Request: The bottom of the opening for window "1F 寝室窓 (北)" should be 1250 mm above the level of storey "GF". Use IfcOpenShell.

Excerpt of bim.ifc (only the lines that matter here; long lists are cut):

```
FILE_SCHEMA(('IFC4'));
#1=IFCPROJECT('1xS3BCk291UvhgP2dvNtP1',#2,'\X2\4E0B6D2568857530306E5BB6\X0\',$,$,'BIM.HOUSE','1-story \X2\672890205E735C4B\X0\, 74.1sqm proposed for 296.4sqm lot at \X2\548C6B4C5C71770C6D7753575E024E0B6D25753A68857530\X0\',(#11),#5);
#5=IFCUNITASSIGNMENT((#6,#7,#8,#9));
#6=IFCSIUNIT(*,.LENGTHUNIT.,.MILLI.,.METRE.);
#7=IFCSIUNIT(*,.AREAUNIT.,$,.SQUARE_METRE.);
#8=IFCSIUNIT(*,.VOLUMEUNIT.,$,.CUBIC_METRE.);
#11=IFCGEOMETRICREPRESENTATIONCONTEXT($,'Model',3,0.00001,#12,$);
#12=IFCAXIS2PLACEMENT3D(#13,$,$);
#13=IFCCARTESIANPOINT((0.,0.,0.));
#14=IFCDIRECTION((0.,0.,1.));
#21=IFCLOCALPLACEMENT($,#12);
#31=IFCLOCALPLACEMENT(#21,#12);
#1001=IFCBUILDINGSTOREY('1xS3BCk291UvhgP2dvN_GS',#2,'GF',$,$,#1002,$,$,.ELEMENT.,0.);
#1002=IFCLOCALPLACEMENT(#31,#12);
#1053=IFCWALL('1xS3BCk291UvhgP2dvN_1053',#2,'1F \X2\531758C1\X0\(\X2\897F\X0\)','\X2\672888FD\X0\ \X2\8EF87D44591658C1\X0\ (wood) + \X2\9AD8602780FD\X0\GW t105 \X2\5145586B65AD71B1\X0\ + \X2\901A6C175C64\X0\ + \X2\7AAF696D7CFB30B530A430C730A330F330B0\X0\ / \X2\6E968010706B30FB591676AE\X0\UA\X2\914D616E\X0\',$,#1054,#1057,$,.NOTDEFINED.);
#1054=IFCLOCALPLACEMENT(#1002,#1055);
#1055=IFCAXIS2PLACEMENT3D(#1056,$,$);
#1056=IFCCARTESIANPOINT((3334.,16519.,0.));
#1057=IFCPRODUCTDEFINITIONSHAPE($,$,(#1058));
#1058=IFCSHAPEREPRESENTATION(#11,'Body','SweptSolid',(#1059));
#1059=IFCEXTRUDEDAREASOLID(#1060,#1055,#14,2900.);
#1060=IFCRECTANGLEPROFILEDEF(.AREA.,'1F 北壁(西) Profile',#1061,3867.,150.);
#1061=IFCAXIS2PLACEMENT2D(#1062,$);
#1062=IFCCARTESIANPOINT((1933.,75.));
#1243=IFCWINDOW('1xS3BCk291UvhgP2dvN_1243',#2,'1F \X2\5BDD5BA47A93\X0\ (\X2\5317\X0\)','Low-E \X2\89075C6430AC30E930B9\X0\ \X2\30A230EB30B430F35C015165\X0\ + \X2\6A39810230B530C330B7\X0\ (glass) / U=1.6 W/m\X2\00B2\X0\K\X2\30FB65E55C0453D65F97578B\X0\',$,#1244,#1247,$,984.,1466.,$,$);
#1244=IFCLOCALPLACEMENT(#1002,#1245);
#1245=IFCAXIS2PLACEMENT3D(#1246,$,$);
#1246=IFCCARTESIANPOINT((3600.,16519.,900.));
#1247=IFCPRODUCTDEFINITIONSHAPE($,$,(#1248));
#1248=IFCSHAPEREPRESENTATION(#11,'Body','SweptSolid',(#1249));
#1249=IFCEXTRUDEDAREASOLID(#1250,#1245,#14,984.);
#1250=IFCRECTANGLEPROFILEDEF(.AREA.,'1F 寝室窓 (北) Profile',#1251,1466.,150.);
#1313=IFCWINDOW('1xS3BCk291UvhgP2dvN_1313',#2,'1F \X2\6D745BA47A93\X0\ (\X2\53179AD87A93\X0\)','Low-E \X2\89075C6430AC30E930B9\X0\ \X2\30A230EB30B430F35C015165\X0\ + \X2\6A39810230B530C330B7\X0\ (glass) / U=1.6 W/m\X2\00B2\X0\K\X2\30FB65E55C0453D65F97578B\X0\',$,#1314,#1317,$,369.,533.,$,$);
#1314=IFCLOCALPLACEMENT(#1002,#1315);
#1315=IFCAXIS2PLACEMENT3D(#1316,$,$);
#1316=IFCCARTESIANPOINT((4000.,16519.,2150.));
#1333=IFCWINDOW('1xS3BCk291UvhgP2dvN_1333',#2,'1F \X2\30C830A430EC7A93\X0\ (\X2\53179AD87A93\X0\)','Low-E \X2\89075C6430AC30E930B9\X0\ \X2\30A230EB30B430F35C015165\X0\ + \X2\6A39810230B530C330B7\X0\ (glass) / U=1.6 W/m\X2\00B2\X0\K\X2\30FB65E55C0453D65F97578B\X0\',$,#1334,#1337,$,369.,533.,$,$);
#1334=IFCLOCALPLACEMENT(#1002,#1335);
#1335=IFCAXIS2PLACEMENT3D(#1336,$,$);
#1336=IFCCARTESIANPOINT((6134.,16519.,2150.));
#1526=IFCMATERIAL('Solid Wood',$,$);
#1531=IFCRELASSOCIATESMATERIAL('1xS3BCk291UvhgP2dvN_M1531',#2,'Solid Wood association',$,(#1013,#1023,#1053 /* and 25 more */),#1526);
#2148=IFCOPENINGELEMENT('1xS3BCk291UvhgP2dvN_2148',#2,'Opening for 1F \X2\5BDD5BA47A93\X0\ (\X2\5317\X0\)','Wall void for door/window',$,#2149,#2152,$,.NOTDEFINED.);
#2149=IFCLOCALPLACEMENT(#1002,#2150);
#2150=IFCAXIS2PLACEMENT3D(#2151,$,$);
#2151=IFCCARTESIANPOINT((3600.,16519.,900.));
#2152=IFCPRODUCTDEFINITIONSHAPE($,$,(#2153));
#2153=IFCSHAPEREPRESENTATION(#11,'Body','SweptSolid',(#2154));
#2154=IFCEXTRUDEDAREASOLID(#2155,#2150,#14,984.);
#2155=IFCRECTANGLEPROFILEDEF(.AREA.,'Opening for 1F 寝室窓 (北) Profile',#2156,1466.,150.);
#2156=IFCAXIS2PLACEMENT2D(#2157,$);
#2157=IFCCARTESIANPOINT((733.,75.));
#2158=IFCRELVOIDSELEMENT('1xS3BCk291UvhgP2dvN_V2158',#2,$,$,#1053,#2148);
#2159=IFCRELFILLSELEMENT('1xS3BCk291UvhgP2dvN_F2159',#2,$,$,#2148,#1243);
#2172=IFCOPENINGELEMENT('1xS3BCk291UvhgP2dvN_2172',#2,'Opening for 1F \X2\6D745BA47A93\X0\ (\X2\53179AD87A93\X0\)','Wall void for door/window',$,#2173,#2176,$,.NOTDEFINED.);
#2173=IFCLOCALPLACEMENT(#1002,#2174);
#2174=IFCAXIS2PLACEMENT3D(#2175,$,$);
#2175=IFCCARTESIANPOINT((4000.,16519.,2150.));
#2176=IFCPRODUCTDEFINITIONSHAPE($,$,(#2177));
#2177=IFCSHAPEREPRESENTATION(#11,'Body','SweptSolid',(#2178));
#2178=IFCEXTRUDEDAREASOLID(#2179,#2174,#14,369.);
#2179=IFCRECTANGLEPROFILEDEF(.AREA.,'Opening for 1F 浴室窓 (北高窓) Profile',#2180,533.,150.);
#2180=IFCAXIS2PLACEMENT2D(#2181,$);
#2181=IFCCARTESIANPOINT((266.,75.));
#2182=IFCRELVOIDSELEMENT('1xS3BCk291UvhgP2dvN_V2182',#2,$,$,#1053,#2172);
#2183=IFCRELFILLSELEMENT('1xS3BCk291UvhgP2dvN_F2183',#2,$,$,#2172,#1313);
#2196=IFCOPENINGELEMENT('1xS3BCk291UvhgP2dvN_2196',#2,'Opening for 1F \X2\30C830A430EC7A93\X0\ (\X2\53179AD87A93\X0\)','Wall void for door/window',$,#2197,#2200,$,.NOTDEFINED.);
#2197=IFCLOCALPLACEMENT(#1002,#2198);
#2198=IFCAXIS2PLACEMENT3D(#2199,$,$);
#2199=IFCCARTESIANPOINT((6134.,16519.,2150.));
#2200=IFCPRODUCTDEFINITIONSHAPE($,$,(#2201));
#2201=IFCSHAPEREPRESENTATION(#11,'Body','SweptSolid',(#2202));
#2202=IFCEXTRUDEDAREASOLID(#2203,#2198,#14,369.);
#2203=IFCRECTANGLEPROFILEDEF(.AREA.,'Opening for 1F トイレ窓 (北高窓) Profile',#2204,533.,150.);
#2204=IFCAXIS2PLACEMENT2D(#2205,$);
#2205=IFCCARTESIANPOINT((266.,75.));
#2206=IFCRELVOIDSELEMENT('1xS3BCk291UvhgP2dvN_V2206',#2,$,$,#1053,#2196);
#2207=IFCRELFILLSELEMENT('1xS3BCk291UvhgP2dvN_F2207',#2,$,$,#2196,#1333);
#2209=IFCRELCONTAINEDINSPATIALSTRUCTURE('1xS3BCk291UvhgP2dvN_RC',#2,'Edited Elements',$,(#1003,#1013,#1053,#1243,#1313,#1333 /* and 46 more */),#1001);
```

```python
import numpy as np
import ifcopenshell
import ifcopenshell.api.geometry
import ifcopenshell.geom
import ifcopenshell.util.element
import ifcopenshell.util.placement
import ifcopenshell.util.shape
import ifcopenshell.util.unit

model = ifcopenshell.open("bim.ifc")
unit_scale = ifcopenshell.util.unit.calculate_unit_scale(model)

window = model.by_guid("1xS3BCk291UvhgP2dvN_1243")
opening = window.FillsVoids[0].RelatingOpeningElement
storey = ifcopenshell.util.element.get_container(window, ifc_class="IfcBuildingStorey")
level = ifcopenshell.util.placement.get_local_placement(storey.ObjectPlacement)[2, 3]

# The opening's origin need not be at the sill, so measure its lowest point.
shape = ifcopenshell.geom.create_shape(ifcopenshell.geom.settings(), opening)
bottom = ifcopenshell.util.shape.get_shape_bottom_elevation(shape, shape.geometry) / unit_scale
dz = level + 1.25 / unit_scale - bottom

shift = np.array([0.0, 0.0, dz])
# The window is not placed relative to its opening, so move both.
for product in (opening, window):
    matrix = ifcopenshell.util.placement.get_local_placement(product.ObjectPlacement)
    matrix[:3, 3] += shift
    ifcopenshell.api.geometry.edit_object_placement(model, product=product, matrix=matrix, is_si=False)

print(f"moved by {dz * unit_scale:+.3f} m")

model.write("bim_updated.ifc")
```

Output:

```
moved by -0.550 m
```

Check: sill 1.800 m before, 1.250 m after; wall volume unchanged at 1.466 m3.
